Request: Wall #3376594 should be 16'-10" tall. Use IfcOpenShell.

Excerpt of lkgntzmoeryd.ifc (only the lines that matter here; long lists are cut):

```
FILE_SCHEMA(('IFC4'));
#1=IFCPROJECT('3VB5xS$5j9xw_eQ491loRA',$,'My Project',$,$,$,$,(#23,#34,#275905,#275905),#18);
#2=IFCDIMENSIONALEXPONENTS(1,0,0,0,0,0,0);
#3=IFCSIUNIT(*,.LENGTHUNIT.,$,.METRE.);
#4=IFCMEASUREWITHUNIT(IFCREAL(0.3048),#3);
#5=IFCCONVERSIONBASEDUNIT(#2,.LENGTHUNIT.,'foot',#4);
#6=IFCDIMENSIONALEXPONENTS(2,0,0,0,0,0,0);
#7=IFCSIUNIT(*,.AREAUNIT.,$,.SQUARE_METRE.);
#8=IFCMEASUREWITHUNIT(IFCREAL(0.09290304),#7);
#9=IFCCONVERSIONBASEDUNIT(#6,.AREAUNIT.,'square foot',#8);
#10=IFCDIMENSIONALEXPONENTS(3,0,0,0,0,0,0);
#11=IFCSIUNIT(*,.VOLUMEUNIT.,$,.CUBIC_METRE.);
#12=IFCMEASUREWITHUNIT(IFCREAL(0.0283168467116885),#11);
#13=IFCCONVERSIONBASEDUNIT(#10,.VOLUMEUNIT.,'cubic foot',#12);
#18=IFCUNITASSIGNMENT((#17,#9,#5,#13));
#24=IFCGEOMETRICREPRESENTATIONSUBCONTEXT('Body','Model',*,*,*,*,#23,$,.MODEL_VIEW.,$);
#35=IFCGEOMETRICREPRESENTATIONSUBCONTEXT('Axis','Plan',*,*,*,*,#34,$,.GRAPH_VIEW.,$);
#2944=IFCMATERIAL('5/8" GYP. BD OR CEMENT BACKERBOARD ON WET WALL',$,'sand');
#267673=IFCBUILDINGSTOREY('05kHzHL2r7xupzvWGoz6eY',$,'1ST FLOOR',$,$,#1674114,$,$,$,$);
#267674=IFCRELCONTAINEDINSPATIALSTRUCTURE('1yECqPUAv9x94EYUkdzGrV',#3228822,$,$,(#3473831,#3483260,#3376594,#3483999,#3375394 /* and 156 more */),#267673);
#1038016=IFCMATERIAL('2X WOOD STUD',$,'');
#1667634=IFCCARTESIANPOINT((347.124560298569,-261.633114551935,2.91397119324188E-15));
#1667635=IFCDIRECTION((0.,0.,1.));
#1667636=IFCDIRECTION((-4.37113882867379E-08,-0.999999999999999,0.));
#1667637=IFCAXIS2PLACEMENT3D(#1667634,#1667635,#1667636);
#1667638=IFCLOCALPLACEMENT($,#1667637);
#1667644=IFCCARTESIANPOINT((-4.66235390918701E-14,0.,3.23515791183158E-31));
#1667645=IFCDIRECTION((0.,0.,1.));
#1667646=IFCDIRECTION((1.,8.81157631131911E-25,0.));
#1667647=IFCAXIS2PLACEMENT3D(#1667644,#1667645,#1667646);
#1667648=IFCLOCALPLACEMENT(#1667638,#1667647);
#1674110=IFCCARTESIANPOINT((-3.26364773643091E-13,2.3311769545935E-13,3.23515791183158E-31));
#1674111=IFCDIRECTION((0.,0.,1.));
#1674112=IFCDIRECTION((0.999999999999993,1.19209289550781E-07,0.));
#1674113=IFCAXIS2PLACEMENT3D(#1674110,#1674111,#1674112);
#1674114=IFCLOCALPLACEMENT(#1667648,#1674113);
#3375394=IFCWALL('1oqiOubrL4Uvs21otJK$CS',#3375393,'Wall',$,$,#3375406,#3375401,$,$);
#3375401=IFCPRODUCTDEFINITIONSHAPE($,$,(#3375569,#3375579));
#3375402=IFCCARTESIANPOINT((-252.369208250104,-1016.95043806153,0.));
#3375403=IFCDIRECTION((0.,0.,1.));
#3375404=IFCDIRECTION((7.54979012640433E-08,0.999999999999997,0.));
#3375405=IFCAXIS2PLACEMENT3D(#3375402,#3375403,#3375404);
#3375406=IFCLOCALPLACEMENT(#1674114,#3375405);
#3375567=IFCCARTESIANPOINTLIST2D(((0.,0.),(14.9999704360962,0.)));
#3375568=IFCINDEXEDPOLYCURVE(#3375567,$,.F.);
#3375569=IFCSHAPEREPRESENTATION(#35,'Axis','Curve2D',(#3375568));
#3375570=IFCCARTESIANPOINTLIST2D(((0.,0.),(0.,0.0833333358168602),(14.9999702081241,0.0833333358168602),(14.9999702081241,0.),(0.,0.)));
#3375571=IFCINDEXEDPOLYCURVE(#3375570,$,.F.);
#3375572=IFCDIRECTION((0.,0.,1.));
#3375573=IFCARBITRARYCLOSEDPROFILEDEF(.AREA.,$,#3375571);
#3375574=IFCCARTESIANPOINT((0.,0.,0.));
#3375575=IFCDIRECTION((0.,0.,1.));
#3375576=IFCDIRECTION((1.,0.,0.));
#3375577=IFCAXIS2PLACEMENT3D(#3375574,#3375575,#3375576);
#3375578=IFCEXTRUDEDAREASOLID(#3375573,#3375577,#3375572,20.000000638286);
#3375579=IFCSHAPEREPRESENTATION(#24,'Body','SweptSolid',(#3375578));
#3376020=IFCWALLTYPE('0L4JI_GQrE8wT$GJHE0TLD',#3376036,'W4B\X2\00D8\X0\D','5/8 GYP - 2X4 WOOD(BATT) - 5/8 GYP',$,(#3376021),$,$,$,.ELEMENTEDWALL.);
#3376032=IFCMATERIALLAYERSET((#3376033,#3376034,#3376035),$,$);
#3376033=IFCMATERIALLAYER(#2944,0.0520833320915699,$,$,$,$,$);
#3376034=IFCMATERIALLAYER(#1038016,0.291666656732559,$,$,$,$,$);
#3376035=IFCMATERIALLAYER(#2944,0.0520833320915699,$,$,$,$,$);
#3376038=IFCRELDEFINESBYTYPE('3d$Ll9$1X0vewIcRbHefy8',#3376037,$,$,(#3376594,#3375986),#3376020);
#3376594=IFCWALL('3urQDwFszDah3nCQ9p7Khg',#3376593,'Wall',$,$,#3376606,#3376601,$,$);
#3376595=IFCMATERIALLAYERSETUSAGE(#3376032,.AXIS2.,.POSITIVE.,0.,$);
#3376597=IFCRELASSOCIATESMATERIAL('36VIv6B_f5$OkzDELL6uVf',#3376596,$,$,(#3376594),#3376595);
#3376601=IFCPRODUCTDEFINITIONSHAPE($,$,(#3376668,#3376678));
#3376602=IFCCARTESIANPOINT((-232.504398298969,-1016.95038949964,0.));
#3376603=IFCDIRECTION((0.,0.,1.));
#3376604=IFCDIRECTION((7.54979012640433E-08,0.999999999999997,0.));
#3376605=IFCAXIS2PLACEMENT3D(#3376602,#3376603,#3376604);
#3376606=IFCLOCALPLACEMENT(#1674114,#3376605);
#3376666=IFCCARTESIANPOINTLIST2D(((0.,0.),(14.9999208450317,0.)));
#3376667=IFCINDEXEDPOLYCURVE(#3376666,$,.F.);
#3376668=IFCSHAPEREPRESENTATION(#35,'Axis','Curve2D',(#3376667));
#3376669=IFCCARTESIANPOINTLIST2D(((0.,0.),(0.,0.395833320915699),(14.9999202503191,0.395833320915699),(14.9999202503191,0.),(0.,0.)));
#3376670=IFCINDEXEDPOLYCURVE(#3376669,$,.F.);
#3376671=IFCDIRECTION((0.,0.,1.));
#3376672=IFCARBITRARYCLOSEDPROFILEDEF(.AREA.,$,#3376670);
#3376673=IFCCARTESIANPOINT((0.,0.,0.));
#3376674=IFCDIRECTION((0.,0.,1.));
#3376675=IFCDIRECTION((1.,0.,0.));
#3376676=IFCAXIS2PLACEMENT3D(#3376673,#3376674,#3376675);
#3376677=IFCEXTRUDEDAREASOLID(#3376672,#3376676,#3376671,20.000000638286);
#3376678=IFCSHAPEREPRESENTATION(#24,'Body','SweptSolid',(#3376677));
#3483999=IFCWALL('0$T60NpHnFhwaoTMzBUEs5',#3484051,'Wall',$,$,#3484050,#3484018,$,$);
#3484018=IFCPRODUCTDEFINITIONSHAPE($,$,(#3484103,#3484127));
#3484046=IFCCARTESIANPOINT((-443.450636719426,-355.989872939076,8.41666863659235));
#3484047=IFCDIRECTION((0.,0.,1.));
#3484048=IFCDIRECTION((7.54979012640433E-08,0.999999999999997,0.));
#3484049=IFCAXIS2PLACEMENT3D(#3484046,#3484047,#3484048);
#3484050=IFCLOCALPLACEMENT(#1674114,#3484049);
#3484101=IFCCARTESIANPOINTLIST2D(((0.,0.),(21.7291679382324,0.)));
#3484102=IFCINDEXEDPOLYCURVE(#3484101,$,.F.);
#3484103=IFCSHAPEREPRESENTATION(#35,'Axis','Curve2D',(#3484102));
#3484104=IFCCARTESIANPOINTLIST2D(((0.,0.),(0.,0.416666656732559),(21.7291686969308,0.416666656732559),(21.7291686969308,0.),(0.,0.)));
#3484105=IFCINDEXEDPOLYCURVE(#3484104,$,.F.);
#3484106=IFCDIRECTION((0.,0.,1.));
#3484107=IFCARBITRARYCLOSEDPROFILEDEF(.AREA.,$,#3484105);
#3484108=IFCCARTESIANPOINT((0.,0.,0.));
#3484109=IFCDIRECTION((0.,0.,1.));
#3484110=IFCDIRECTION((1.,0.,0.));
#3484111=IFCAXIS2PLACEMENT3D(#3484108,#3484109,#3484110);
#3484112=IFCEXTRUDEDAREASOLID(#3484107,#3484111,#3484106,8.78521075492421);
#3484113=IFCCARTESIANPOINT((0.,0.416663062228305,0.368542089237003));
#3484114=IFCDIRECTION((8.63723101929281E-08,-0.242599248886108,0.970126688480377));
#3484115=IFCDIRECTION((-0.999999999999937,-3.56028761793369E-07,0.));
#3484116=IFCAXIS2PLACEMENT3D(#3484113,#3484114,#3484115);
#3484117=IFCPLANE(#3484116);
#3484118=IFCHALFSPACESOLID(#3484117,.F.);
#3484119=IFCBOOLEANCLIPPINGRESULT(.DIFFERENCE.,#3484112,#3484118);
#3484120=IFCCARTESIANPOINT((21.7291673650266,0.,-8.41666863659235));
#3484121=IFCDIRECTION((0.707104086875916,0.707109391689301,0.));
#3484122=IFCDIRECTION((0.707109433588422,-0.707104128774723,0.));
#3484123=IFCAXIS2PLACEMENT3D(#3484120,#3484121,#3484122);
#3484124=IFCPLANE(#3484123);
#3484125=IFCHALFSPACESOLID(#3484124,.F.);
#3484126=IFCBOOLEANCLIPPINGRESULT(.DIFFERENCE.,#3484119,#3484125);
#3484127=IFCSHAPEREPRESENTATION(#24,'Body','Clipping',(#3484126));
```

```python
import ifcopenshell
import ifcopenshell.geom
import ifcopenshell.util.representation
import ifcopenshell.util.shape
import ifcopenshell.util.unit

model = ifcopenshell.open("lkgntzmoeryd.ifc")
unit_scale = ifcopenshell.util.unit.calculate_unit_scale(model)
settings = ifcopenshell.geom.settings()


def volume(element):
    """Net volume in cubic metres, openings subtracted."""
    shape = ifcopenshell.geom.create_shape(settings, element)
    return ifcopenshell.util.shape.get_volume(shape.geometry)


wall = model.by_guid("3urQDwFszDah3nCQ9p7Khg")
before = volume(wall)

body = ifcopenshell.util.representation.get_representation(wall, "Model", "Body")
solid = body.Items[0]
old_height = solid.Depth
solid.Depth = 202 * 0.0254 / unit_scale
after = volume(wall)

print(f"height {old_height:g} -> {solid.Depth:g}, volume {before:.3f} -> {after:.3f} m3")

model.write("lkgntzmoeryd_updated.ifc")
```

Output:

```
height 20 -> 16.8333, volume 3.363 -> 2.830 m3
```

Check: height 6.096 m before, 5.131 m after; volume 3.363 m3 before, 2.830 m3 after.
